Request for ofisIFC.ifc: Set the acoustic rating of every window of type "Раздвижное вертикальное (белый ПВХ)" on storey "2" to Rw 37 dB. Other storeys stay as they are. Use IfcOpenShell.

First a look at what the model holds.

```python
import ifcopenshell
import ifcopenshell.util.element

model = ifcopenshell.open("ofisIFC.ifc")
print(model.schema)
storey = next(s for s in model.by_type("IfcBuildingStorey") if s.Name == "2")
windows = [e for e in ifcopenshell.util.element.get_decomposition(storey) if e.is_a("IfcWindow")]
seen = {}
for e in windows:
    element_type = ifcopenshell.util.element.get_type(e)
    key = (element_type.Name if element_type != e and element_type else None, ifcopenshell.util.element.get_pset(e, "Pset_WindowCommon", "AcousticRating"))
    seen[key] = seen.get(key, 0) + 1
for (name, value), count in sorted(seen.items(), key=str):
    print(count, "x", name, "|", value)
```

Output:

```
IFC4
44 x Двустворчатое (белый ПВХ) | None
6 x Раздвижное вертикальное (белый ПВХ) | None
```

```python
import ifcopenshell
import ifcopenshell.api.pset
import ifcopenshell.util.element

model = ifcopenshell.open("ofisIFC.ifc")

storey = next(s for s in model.by_type("IfcBuildingStorey") if s.Name == "2")
windows = [e for e in ifcopenshell.util.element.get_decomposition(storey) if e.is_a("IfcWindow")]

count = 0
for e in windows:
    element_type = ifcopenshell.util.element.get_type(e)
    if element_type in (None, e) or element_type.Name != "Раздвижное вертикальное (белый ПВХ)":
        continue
    # add_pset returns the element's existing set when there is one.
    pset = ifcopenshell.api.pset.add_pset(model, product=e, name="Pset_WindowCommon")
    ifcopenshell.api.pset.edit_pset(model, pset=pset, properties={"AcousticRating": "Rw 37 dB"})
    count += 1

print(count, "windows updated")

model.write("ofisIFC_rev.ifc")
```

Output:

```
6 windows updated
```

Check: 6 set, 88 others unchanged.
